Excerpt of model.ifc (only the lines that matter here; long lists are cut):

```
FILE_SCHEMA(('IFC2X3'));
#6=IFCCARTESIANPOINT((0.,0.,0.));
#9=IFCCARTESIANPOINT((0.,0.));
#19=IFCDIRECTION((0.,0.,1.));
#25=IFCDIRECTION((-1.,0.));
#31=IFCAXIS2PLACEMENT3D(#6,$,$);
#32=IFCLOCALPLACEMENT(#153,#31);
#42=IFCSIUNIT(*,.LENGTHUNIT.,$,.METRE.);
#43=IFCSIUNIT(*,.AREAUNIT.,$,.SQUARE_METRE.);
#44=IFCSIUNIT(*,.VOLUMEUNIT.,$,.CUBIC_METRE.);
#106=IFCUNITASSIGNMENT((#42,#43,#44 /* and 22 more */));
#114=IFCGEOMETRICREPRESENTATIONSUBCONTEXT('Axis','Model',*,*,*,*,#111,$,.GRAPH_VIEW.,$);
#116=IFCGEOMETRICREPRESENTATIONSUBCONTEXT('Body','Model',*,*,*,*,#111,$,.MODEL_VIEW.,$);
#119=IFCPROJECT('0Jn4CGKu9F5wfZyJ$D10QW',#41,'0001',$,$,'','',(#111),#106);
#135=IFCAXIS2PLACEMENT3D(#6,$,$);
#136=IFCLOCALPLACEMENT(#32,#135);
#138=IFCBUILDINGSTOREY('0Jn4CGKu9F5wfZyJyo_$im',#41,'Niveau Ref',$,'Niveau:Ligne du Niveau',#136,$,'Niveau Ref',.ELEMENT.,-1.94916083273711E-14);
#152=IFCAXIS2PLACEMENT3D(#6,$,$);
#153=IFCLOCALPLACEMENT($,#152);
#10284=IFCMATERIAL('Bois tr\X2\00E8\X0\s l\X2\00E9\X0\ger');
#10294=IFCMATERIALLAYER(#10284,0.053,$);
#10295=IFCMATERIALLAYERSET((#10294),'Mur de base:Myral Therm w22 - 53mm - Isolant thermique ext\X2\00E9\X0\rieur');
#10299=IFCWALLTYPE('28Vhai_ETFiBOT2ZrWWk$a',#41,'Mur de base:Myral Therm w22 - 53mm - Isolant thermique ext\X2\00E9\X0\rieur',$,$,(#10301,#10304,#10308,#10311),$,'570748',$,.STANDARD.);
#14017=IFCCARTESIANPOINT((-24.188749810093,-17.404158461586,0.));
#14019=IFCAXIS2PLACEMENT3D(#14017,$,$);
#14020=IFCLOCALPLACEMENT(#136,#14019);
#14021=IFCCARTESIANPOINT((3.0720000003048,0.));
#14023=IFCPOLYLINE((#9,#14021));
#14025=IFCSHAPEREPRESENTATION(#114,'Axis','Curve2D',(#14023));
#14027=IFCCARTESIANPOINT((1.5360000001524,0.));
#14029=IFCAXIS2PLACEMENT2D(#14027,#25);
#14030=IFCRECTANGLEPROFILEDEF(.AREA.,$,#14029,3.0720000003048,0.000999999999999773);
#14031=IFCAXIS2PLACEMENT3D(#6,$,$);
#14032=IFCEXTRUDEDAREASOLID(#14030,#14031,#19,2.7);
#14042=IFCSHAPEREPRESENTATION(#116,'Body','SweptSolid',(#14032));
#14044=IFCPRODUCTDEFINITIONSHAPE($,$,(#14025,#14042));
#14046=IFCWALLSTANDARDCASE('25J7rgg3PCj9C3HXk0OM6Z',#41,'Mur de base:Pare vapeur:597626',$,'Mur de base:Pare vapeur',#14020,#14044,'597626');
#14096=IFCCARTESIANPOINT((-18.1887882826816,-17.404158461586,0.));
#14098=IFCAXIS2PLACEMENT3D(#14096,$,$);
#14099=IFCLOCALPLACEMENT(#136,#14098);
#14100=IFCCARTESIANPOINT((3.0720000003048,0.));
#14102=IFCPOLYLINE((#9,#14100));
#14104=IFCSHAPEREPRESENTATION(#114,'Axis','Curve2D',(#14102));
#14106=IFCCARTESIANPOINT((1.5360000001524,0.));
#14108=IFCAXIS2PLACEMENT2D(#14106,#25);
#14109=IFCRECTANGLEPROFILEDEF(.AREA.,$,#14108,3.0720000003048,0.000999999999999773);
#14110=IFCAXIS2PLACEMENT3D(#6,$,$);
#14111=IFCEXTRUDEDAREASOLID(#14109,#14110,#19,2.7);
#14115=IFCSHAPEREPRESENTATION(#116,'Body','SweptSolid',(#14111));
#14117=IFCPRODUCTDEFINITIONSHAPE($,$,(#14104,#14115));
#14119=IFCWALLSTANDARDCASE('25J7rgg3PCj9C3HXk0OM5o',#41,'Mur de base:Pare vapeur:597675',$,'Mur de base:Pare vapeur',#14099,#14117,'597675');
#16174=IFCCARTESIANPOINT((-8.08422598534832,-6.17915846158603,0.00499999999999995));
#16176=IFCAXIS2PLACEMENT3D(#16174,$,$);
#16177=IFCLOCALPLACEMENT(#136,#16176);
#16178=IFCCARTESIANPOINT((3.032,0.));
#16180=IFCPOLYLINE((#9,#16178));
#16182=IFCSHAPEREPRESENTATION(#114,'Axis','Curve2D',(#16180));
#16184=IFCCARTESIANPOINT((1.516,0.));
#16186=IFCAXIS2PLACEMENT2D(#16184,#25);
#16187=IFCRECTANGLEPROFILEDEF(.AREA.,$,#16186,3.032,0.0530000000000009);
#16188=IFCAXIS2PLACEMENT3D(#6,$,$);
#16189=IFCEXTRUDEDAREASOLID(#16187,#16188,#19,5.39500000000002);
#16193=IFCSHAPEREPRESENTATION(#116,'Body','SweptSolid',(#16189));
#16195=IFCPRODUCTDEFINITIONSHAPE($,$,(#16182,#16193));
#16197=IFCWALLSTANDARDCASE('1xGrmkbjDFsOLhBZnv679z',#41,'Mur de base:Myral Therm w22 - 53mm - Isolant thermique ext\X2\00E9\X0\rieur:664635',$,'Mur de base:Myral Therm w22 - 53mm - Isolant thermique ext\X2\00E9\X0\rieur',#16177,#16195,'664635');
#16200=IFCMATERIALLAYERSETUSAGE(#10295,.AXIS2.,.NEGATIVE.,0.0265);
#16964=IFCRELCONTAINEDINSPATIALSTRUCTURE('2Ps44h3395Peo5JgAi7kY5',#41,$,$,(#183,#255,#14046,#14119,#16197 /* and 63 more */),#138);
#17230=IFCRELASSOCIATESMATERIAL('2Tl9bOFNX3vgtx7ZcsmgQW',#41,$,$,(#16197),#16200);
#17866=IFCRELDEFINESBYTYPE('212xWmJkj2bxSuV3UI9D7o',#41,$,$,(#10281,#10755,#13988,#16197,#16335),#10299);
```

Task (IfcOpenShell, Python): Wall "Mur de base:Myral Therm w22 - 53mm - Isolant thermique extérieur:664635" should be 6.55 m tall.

```python
import ifcopenshell
import ifcopenshell.geom
import ifcopenshell.util.representation
import ifcopenshell.util.shape
import ifcopenshell.util.unit

model = ifcopenshell.open("model.ifc")
unit_scale = ifcopenshell.util.unit.calculate_unit_scale(model)
settings = ifcopenshell.geom.settings()


def volume(element):
    """Net volume in cubic metres, openings subtracted."""
    shape = ifcopenshell.geom.create_shape(settings, element)
    return ifcopenshell.util.shape.get_volume(shape.geometry)


wall = model.by_id(16197)
before = volume(wall)

body = ifcopenshell.util.representation.get_representation(wall, "Model", "Body")
solid = body.Items[0]
old_height = solid.Depth
solid.Depth = 6.55 / unit_scale
after = volume(wall)

print(f"height {old_height:g} -> {solid.Depth:g}, volume {before:.3f} -> {after:.3f} m3")

model.write("model_edited.ifc")
```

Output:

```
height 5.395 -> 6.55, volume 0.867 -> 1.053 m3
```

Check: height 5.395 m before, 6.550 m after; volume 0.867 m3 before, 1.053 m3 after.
